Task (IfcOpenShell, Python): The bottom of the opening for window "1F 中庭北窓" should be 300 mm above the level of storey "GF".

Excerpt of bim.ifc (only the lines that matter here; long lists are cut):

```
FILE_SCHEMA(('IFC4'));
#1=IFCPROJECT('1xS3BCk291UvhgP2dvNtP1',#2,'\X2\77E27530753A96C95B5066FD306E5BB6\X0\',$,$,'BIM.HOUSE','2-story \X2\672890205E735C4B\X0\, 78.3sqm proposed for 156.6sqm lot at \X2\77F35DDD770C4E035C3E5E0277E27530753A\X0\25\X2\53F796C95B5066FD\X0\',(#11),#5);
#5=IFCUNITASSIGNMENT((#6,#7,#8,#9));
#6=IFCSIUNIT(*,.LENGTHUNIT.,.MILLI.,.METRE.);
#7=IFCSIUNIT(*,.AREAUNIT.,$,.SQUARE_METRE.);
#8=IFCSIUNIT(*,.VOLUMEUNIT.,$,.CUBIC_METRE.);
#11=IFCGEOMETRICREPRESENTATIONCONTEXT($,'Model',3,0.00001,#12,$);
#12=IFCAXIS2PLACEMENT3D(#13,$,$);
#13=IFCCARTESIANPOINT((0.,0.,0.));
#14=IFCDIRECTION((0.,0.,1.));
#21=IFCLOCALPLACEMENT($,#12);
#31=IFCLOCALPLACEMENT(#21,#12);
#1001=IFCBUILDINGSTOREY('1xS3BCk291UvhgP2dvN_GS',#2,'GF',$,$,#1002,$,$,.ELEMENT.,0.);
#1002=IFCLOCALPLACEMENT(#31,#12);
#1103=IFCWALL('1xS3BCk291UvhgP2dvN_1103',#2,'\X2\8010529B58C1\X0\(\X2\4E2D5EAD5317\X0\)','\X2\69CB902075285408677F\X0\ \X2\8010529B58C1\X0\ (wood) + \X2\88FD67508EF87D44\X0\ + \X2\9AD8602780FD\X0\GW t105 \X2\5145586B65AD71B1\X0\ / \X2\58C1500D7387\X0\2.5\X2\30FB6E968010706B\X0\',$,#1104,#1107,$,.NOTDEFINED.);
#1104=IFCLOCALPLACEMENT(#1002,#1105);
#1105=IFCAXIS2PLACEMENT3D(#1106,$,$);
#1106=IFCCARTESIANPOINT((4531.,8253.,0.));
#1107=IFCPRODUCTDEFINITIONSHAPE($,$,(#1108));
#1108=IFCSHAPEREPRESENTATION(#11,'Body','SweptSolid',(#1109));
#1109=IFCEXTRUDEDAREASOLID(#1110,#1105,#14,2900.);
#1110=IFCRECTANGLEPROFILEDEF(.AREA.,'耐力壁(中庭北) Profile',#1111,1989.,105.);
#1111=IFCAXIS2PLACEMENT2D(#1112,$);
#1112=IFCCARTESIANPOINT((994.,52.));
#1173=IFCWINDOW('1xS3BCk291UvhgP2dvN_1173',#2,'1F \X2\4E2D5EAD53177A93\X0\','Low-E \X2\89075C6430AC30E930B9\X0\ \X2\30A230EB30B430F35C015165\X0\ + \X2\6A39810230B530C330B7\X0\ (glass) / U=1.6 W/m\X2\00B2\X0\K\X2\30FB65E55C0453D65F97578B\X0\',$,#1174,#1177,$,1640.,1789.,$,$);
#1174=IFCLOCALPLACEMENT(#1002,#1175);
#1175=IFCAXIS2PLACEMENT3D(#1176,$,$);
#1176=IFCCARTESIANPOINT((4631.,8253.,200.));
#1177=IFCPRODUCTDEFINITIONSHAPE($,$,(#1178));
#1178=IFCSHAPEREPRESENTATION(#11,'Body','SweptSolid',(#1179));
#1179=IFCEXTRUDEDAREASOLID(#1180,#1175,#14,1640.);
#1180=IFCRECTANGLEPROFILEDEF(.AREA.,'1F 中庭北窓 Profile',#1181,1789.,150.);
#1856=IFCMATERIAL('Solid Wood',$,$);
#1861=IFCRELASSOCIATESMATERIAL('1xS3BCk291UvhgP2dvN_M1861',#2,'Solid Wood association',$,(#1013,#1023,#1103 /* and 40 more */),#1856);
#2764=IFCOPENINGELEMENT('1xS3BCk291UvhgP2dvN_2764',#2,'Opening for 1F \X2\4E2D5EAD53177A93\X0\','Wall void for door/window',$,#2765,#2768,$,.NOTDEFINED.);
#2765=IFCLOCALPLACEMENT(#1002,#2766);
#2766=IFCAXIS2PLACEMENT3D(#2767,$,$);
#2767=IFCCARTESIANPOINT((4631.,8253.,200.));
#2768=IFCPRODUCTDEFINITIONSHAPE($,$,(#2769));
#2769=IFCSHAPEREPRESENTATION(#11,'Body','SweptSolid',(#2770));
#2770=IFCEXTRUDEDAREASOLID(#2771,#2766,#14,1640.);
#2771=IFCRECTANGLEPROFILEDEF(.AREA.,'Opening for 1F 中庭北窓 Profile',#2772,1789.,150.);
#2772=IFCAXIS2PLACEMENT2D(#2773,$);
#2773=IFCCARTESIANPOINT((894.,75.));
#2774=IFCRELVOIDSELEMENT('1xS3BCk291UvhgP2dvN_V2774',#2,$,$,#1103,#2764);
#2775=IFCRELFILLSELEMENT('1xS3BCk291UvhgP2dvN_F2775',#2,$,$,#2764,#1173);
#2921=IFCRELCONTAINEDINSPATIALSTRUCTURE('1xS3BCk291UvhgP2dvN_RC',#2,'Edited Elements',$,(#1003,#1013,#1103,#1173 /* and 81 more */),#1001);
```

```python
import numpy as np
import ifcopenshell
import ifcopenshell.api.geometry
import ifcopenshell.geom
import ifcopenshell.util.element
import ifcopenshell.util.placement
import ifcopenshell.util.shape
import ifcopenshell.util.unit

model = ifcopenshell.open("bim.ifc")
unit_scale = ifcopenshell.util.unit.calculate_unit_scale(model)

window = model.by_id(1173)
opening = window.FillsVoids[0].RelatingOpeningElement
storey = ifcopenshell.util.element.get_container(window, ifc_class="IfcBuildingStorey")
level = ifcopenshell.util.placement.get_local_placement(storey.ObjectPlacement)[2, 3]

# The opening's origin need not be at the sill, so measure its lowest point.
shape = ifcopenshell.geom.create_shape(ifcopenshell.geom.settings(), opening)
bottom = ifcopenshell.util.shape.get_shape_bottom_elevation(shape, shape.geometry) / unit_scale
dz = level + 300.0 - bottom

shift = np.array([0.0, 0.0, dz])
# The window is not placed relative to its opening, so move both.
for product in (opening, window):
    matrix = ifcopenshell.util.placement.get_local_placement(product.ObjectPlacement)
    matrix[:3, 3] += shift
    ifcopenshell.api.geometry.edit_object_placement(model, product=product, matrix=matrix, is_si=False)

print(f"moved by {dz * unit_scale:+.3f} m")

model.write("bim-out.ifc")
```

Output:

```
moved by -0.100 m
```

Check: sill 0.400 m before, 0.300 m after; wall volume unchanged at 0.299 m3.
